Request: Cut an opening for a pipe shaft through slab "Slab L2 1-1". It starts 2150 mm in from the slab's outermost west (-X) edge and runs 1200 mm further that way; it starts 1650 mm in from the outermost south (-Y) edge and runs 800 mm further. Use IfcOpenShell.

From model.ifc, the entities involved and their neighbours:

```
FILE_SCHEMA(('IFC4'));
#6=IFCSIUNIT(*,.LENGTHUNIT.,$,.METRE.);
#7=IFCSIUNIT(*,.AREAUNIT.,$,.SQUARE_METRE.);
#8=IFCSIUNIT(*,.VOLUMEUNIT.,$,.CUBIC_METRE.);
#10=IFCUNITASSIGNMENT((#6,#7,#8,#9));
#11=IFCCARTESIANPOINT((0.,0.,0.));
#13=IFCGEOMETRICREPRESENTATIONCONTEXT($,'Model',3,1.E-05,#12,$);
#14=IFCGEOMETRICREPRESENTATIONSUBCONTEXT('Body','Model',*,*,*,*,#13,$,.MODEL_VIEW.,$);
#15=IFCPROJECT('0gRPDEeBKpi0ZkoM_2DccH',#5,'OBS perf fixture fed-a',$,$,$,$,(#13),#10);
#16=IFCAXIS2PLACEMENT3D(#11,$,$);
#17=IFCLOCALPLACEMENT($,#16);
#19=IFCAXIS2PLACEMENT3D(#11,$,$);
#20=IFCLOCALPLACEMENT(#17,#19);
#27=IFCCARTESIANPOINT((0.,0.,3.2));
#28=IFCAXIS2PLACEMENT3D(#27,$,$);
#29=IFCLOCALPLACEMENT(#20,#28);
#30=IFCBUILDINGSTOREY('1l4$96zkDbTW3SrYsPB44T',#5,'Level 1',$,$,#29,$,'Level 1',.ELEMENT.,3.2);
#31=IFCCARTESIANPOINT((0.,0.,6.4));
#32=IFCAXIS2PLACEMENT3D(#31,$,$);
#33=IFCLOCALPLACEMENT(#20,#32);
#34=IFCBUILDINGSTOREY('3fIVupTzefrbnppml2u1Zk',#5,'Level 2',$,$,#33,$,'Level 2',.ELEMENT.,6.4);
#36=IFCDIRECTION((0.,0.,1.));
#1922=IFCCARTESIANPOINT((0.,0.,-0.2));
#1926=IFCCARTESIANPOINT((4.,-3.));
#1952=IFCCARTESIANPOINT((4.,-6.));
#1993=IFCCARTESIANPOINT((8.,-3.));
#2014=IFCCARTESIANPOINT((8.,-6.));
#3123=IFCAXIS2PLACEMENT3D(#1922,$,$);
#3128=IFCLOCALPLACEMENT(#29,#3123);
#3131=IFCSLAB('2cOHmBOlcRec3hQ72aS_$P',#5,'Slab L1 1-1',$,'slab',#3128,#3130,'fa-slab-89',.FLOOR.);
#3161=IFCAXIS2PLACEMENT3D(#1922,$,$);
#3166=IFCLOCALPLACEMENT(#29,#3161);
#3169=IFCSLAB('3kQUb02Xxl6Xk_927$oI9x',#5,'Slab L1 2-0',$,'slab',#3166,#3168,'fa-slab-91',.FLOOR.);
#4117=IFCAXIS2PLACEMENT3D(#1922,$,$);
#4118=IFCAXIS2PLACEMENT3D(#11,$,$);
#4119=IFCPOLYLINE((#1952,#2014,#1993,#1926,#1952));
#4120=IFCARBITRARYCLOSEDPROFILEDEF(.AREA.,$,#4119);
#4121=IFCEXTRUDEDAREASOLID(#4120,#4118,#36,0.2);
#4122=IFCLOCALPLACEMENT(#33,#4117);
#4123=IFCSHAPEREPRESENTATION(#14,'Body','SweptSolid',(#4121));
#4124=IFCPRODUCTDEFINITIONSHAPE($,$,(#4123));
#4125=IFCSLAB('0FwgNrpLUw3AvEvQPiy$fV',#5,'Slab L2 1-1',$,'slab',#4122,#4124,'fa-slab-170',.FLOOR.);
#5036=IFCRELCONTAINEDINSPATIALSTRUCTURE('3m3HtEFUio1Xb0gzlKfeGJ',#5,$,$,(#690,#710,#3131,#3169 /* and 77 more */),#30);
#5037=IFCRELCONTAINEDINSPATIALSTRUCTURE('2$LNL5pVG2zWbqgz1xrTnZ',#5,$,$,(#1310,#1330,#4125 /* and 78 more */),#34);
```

```python
import numpy as np
import ifcopenshell
import ifcopenshell.api.feature
import ifcopenshell.api.geometry
import ifcopenshell.api.root
import ifcopenshell.geom
import ifcopenshell.util.placement
import ifcopenshell.util.representation
import ifcopenshell.util.shape
import ifcopenshell.util.unit

model = ifcopenshell.open("model.ifc")
unit_scale = ifcopenshell.util.unit.calculate_unit_scale(model)
settings = ifcopenshell.geom.settings()


def volume(element):
    """Net volume in cubic metres, openings subtracted."""
    shape = ifcopenshell.geom.create_shape(settings, element)
    return ifcopenshell.util.shape.get_volume(shape.geometry)


slab = model.by_id(4125)
before = volume(slab)

# Extent in the slab's own axes, in metres. The edges named are its -X and -Y sides.
slab_shape = ifcopenshell.geom.create_shape(settings, slab)
vertices = ifcopenshell.util.shape.get_vertices(slab_shape.geometry)
x_min, y_min, bottom = vertices.min(axis=0)
top = vertices[:, 2].max()

opening = ifcopenshell.api.root.create_entity(model, ifc_class="IfcOpeningElement", name="Pipe shaft opening", predefined_type="OPENING")
context = ifcopenshell.util.representation.get_context(model, "Model", "Body", "MODEL_VIEW")
width, depth = 1.2, 0.8
outline = [(0.0, 0.0), (width, 0.0), (width, depth), (0.0, depth), (0.0, 0.0)]
# Overshoot both faces by 50 mm so the cut is clean.
shape = ifcopenshell.api.geometry.add_slab_representation(
    model, context=context, depth=top - bottom + 0.1, polyline=outline
)
ifcopenshell.api.geometry.assign_representation(model, product=opening, representation=shape)

matrix = ifcopenshell.util.placement.get_local_placement(slab.ObjectPlacement)
matrix[:, 3] = matrix @ np.append(np.array([x_min + 2.15, y_min + 1.65, bottom - 0.05]) / unit_scale, 1.0)
ifcopenshell.api.geometry.edit_object_placement(model, product=opening, matrix=matrix, is_si=False)
ifcopenshell.api.feature.add_feature(model, feature=opening, element=slab)

after = volume(slab)

print(f"slab volume {before:.3f} -> {after:.3f} m3")

model.write("model_v2.ifc")
```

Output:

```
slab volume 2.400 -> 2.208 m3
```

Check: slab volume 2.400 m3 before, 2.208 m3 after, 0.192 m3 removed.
